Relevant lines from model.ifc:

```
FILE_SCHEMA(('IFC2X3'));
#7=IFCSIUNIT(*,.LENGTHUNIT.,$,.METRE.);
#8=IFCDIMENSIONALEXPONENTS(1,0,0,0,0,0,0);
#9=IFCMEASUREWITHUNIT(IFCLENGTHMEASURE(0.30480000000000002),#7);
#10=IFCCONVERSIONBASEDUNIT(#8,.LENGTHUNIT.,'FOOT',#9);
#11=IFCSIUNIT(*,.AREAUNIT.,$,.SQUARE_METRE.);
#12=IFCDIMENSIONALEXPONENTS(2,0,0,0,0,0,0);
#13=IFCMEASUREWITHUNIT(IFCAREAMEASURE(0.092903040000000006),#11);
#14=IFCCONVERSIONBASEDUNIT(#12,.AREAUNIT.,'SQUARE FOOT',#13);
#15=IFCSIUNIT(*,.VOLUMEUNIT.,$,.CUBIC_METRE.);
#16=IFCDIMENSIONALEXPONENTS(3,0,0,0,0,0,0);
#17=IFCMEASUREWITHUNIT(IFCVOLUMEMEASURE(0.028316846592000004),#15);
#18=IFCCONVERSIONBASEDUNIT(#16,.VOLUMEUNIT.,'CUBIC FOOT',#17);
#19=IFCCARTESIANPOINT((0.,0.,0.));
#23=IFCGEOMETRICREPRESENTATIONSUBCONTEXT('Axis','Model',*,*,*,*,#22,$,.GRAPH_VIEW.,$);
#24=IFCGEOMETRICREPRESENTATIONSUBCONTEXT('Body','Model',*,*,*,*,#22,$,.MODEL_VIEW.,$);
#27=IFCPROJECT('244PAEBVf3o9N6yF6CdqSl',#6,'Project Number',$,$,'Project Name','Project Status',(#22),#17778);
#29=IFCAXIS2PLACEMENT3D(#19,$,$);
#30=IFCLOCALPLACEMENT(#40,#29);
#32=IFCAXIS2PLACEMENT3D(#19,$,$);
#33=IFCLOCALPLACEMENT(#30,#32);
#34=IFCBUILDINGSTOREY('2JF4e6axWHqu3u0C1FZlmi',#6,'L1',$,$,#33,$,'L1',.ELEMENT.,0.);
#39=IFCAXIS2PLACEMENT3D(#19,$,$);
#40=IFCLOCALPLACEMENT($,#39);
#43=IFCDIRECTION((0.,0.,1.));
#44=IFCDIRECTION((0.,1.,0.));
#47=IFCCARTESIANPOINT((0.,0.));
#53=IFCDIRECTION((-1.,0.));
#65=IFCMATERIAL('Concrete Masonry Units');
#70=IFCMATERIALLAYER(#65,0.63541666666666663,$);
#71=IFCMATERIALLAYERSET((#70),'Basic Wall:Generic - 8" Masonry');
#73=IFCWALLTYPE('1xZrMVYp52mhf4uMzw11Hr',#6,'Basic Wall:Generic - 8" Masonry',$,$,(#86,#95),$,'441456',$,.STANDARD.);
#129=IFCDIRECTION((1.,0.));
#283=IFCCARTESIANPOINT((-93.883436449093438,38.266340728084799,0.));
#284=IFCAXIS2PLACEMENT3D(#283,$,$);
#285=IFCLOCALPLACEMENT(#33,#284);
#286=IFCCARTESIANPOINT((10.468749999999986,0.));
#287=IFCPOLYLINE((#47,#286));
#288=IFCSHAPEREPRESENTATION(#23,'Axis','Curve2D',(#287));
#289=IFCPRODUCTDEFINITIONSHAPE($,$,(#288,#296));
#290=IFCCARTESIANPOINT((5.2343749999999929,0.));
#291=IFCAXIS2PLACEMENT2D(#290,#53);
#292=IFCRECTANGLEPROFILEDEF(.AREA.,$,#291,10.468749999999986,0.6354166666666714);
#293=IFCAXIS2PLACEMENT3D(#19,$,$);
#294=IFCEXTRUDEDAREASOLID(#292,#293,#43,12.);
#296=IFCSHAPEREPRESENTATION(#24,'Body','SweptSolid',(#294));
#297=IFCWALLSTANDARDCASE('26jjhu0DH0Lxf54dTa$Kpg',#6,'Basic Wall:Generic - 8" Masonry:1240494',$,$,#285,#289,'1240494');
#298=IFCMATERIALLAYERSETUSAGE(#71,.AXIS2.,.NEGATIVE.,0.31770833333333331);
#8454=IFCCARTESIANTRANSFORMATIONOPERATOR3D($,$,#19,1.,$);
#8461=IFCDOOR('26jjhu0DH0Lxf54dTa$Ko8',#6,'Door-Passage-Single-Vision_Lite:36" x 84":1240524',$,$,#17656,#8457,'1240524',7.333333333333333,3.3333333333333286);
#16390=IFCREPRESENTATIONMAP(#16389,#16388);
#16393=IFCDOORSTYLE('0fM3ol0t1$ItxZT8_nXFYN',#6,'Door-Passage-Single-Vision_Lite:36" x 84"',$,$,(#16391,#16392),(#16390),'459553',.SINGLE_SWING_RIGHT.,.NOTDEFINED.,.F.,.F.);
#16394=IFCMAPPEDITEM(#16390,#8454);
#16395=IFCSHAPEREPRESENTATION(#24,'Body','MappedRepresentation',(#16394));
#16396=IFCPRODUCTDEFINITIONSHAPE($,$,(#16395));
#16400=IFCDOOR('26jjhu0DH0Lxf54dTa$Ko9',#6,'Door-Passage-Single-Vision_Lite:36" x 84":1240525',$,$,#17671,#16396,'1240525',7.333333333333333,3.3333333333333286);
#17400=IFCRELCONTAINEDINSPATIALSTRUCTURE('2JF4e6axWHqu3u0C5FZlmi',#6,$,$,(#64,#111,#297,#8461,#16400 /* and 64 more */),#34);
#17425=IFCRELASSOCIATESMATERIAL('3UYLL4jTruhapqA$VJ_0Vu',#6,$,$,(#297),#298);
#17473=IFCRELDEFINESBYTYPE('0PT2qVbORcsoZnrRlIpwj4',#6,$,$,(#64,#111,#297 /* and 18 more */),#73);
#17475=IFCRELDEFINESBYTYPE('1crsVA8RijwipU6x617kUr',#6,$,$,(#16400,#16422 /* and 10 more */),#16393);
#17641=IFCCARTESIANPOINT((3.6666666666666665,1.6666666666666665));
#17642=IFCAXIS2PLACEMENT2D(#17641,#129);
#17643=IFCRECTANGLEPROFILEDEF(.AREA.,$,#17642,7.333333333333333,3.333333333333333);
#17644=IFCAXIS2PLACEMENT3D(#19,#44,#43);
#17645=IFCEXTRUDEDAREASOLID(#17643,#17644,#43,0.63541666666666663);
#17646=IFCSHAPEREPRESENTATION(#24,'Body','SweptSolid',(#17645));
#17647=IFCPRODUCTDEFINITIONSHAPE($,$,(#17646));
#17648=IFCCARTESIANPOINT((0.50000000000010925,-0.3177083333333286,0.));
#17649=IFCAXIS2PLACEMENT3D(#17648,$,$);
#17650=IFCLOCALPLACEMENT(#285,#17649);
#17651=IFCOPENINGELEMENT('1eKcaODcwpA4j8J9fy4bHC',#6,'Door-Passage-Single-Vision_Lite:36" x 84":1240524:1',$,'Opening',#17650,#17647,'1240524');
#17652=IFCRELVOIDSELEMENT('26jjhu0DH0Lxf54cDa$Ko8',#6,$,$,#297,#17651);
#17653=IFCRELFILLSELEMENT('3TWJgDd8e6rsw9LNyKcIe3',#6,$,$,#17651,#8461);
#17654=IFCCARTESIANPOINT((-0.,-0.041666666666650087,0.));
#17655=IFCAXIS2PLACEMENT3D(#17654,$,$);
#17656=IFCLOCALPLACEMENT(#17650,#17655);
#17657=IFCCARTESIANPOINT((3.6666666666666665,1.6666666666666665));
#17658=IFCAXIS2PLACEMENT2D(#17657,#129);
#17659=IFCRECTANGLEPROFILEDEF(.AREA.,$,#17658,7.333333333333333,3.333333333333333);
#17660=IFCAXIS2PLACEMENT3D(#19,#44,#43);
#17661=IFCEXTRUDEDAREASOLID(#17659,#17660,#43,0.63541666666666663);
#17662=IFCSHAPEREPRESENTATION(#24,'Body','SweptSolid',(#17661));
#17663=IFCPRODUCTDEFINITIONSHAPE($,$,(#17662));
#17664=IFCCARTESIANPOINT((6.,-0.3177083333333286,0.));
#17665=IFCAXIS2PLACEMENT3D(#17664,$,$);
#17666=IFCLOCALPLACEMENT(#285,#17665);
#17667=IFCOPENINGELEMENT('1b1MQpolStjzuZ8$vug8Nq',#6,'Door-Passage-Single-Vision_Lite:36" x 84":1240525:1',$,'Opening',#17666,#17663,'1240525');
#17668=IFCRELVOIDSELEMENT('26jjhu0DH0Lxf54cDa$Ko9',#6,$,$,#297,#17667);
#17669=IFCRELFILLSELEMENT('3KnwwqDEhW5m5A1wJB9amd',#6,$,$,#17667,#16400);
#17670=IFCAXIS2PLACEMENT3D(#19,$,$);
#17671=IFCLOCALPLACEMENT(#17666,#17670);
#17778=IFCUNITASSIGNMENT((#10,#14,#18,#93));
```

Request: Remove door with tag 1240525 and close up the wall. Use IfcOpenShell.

```python
import ifcopenshell
import ifcopenshell.api.feature
import ifcopenshell.api.root
import ifcopenshell.geom
import ifcopenshell.util.shape

model = ifcopenshell.open("model.ifc")
settings = ifcopenshell.geom.settings()


def volume(element):
    """Net volume in cubic metres, openings subtracted."""
    shape = ifcopenshell.geom.create_shape(settings, element)
    return ifcopenshell.util.shape.get_volume(shape.geometry)


door = model.by_id(16400)
opening = door.FillsVoids[0].RelatingOpeningElement
wall = opening.VoidsElements[0].RelatingBuildingElement
before = volume(wall)

ifcopenshell.api.root.remove_product(model, product=door)
ifcopenshell.api.feature.remove_feature(model, feature=opening)

after = volume(wall)

print(f"wall volume {before:.3f} -> {after:.3f} m3")

model.write("model_v2.ifc")
```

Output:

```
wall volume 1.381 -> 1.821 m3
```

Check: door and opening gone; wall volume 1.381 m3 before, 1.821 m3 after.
